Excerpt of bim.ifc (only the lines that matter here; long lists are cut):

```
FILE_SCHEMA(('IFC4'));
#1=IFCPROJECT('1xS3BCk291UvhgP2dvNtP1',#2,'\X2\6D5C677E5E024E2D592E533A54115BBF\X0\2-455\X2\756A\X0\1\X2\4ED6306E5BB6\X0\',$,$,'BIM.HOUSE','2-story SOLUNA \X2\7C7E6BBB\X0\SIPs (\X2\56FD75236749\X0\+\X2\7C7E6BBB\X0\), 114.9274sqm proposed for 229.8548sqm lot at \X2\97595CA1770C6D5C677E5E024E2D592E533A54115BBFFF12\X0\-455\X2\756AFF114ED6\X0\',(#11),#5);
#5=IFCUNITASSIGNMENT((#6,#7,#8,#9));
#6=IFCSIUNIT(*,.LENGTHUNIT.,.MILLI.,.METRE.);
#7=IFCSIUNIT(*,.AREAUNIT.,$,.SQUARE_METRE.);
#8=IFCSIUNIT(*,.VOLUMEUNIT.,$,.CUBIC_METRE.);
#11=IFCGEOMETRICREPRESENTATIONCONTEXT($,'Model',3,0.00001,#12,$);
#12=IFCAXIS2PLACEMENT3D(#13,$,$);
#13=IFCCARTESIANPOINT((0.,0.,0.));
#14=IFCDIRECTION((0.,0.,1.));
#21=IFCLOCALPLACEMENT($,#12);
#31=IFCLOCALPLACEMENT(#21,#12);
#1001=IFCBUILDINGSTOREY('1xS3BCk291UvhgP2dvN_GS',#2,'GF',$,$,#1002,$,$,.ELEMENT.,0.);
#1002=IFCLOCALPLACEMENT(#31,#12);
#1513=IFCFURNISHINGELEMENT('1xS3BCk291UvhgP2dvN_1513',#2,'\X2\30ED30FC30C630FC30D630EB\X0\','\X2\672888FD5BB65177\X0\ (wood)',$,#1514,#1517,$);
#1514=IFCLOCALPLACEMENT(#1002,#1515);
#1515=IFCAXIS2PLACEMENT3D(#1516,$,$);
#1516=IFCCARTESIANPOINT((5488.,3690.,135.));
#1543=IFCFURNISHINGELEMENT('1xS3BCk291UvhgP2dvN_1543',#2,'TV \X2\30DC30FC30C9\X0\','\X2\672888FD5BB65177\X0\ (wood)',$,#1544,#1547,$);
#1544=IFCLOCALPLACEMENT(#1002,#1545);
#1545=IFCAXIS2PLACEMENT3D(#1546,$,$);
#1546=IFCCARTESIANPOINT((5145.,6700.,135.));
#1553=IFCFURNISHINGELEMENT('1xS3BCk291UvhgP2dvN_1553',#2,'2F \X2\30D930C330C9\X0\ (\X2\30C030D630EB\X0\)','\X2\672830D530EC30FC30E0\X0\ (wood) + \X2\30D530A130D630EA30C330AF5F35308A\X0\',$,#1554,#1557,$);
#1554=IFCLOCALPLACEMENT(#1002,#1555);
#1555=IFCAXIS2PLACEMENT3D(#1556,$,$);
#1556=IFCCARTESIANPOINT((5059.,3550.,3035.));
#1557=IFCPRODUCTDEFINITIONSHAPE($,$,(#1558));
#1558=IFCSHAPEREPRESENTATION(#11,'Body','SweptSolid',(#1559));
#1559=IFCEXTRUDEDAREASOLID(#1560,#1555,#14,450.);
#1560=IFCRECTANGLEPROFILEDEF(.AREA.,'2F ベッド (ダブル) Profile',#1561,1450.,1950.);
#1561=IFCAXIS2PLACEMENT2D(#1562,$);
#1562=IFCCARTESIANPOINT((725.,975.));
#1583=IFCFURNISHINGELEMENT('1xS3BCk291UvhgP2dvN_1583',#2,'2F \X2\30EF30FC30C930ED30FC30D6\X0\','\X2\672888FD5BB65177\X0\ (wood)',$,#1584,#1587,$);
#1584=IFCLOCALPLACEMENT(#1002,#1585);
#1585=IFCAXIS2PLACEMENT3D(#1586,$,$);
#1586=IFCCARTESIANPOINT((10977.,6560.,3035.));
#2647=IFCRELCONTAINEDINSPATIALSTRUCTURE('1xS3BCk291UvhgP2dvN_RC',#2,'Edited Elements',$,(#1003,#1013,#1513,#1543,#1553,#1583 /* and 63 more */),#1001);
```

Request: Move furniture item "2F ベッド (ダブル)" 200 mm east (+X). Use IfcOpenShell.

```python
import ifcopenshell
import ifcopenshell.api.geometry
import ifcopenshell.util.placement
import ifcopenshell.util.unit

model = ifcopenshell.open("bim.ifc")
unit_scale = ifcopenshell.util.unit.calculate_unit_scale(model)

item = model.by_guid("1xS3BCk291UvhgP2dvN_1553")
matrix = ifcopenshell.util.placement.get_local_placement(item.ObjectPlacement)
matrix[0, 3] += 0.2 / unit_scale
ifcopenshell.api.geometry.edit_object_placement(model, product=item, matrix=matrix, is_si=False)

print(ifcopenshell.util.placement.get_local_placement(item.ObjectPlacement).round(3) + 0.0)

model.write("bim_updated.ifc")
```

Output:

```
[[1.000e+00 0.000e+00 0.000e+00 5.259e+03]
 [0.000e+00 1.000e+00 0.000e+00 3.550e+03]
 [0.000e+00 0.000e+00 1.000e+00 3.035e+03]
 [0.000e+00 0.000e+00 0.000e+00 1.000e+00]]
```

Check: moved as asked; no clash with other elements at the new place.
